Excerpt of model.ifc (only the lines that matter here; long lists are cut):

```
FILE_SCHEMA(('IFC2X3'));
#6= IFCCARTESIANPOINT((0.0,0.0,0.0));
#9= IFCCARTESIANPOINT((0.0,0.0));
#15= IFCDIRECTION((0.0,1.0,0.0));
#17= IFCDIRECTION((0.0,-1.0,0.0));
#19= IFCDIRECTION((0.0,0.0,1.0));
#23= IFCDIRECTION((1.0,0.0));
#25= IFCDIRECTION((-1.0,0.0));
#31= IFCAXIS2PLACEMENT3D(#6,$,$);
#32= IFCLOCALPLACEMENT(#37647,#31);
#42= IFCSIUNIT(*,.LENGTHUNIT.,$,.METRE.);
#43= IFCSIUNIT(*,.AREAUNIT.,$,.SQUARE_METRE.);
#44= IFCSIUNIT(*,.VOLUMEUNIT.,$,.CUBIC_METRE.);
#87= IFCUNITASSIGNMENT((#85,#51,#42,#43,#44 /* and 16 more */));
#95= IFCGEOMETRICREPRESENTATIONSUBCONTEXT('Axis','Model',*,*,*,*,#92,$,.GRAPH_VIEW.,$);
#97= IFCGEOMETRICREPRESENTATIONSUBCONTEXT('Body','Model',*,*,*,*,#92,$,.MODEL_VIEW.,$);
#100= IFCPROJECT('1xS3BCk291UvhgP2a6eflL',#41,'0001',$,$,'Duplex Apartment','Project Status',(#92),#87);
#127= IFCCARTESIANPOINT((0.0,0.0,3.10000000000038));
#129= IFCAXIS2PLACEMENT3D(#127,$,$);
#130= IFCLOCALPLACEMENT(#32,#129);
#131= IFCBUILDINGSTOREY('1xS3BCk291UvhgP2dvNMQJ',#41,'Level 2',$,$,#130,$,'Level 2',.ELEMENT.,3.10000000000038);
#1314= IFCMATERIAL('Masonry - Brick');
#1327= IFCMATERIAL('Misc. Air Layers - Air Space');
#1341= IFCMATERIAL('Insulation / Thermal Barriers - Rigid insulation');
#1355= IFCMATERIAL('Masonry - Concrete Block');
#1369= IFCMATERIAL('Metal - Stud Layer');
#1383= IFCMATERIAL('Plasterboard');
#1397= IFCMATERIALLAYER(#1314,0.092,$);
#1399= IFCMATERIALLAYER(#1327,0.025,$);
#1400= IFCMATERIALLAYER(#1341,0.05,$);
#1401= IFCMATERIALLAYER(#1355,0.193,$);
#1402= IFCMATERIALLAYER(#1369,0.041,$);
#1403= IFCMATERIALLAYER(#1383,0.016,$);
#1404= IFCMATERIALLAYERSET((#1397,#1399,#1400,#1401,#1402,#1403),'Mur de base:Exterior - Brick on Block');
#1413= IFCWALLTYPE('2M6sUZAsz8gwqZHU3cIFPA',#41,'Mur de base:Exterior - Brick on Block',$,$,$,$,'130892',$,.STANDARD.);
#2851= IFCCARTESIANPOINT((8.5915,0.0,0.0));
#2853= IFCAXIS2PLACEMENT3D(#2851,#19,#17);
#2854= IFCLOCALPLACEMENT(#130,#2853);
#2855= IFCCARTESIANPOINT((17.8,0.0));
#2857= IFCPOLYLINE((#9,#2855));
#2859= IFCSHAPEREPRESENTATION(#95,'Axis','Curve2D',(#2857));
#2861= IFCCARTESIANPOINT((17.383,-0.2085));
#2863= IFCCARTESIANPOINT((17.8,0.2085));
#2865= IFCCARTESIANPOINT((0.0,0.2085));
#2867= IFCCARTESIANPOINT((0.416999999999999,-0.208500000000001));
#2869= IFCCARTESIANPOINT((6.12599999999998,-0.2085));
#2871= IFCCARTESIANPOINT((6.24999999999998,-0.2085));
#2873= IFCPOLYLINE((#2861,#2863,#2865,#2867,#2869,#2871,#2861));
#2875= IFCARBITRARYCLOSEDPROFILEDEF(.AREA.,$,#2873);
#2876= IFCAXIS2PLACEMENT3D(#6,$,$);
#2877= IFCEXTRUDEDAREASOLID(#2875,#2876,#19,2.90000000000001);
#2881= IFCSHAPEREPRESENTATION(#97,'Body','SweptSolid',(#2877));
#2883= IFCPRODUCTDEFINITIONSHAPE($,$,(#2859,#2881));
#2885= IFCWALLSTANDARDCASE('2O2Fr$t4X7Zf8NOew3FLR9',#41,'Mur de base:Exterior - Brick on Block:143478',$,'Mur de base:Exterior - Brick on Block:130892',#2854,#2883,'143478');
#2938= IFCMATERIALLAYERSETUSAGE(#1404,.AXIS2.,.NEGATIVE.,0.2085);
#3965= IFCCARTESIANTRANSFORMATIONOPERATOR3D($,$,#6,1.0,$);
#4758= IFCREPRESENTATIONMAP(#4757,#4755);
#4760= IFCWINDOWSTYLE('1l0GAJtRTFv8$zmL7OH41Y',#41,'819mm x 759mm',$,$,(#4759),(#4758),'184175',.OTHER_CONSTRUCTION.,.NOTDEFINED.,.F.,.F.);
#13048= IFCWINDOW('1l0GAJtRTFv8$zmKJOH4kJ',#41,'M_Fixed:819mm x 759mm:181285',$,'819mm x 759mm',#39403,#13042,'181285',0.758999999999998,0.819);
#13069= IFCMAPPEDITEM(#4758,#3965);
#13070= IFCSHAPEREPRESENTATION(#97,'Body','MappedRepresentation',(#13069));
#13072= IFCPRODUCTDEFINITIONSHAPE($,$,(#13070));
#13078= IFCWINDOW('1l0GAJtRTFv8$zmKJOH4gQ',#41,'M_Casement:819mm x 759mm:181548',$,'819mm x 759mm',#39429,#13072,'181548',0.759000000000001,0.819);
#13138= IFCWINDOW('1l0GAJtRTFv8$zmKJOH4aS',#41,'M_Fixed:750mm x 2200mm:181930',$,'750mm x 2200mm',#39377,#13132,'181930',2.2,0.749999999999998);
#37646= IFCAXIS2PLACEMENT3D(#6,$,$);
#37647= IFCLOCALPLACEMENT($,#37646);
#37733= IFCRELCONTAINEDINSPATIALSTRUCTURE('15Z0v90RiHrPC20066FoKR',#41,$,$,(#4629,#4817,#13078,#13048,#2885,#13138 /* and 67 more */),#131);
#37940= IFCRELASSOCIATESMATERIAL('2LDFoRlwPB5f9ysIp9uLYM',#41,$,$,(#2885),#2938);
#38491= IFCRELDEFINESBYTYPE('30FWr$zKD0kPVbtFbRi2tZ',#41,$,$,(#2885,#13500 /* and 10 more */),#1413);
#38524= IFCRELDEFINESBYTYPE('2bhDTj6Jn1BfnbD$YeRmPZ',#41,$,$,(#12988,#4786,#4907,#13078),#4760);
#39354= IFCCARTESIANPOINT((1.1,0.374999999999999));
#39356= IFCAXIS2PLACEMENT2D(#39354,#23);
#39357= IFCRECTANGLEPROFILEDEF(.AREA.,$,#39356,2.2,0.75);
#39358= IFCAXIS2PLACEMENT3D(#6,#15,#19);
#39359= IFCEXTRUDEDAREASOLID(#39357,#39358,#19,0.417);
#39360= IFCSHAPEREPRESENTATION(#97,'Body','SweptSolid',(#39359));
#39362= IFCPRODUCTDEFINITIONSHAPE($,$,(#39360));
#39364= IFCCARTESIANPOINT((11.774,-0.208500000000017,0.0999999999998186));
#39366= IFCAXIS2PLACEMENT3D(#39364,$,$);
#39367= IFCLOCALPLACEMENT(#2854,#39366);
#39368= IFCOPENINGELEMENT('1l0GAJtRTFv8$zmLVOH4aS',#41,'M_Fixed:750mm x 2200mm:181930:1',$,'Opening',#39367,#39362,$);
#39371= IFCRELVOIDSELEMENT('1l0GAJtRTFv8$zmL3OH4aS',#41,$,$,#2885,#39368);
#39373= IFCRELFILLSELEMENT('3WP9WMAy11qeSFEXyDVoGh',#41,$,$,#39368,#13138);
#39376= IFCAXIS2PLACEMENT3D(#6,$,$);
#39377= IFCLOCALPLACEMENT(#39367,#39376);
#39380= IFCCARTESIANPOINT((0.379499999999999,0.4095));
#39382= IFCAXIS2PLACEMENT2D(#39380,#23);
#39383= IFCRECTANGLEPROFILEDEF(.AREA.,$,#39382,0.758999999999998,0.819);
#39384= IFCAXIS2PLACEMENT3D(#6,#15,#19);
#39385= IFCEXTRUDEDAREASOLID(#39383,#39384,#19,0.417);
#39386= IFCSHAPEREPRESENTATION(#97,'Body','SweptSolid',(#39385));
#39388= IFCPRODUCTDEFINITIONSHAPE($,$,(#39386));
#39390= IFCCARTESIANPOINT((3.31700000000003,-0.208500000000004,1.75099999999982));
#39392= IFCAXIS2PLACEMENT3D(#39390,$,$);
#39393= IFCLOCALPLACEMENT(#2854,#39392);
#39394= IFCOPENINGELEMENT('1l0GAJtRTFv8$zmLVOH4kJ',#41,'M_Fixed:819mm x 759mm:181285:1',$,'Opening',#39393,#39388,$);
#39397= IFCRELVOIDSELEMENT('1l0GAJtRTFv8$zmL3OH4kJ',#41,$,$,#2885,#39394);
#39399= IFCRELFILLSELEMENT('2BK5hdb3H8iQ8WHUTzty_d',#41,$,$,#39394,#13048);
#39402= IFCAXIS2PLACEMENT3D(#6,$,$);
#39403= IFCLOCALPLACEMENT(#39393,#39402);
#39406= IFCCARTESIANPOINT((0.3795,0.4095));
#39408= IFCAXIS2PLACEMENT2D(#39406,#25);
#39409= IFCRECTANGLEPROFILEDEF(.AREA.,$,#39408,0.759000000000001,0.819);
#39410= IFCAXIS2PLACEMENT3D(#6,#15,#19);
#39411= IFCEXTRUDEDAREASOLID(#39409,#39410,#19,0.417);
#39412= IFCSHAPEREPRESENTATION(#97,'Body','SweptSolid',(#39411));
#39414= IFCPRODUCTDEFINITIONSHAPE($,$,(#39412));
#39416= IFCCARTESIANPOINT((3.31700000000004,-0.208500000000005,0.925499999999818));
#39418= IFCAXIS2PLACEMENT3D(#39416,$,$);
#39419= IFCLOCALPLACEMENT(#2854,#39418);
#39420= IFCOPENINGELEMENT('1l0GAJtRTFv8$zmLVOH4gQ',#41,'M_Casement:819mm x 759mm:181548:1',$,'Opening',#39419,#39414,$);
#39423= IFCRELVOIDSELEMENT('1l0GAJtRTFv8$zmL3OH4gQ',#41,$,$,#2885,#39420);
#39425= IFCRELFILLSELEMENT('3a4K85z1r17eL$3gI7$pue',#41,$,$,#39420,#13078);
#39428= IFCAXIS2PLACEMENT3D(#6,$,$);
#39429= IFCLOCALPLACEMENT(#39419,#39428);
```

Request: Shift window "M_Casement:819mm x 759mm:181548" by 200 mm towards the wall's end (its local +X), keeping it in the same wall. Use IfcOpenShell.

```python
import ifcopenshell
import ifcopenshell.api.geometry
import ifcopenshell.util.placement

model = ifcopenshell.open("model.ifc")

window = model.by_id(13078)
opening = window.FillsVoids[0].RelatingOpeningElement
wall = opening.VoidsElements[0].RelatingBuildingElement

wall_matrix = ifcopenshell.util.placement.get_local_placement(wall.ObjectPlacement)
shift = wall_matrix[:3, 0] * 0.2
before = ifcopenshell.util.placement.get_local_placement(window.ObjectPlacement)[:3, 3].copy()

# The window is placed relative to its opening, so it follows when the opening moves.
matrix = ifcopenshell.util.placement.get_local_placement(opening.ObjectPlacement)
matrix[:3, 3] += shift
ifcopenshell.api.geometry.edit_object_placement(
    model, product=opening, matrix=matrix, is_si=False, should_transform_children=True
)

after = ifcopenshell.util.placement.get_local_placement(window.ObjectPlacement)[:3, 3]
print("window moved by", (after - before).round(3) + 0.0)

model.write("model_updated.ifc")
```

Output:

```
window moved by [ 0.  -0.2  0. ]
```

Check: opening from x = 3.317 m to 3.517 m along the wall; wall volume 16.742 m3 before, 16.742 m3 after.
